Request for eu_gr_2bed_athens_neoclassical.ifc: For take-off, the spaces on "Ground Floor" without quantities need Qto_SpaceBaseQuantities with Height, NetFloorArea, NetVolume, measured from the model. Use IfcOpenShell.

First a look at what the model holds.

```python
import ifcopenshell
import ifcopenshell.util.element
import ifcopenshell.util.unit

model = ifcopenshell.open("eu_gr_2bed_athens_neoclassical.ifc")
print(model.schema)
for unit_type in ("LENGTHUNIT", "AREAUNIT", "VOLUMEUNIT"):
    print(unit_type, ifcopenshell.util.unit.calculate_unit_scale(model, unit_type))
storey = next(s for s in model.by_type("IfcBuildingStorey") if s.Name == "Ground Floor")
spaces = [e for e in ifcopenshell.util.element.get_decomposition(storey) if e.is_a("IfcSpace")]
for e in sorted(spaces, key=lambda e: e.id()):
    print(e.id(), e.is_a(), e.Name, list(ifcopenshell.util.element.get_psets(e, qtos_only=True)), sep=" | ")
```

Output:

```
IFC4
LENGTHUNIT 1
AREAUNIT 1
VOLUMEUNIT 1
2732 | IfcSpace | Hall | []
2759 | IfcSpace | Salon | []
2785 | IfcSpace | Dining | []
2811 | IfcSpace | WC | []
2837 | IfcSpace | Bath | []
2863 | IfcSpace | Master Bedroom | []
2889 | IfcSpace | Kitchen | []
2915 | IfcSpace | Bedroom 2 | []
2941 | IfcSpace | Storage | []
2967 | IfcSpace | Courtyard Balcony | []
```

```python
import ifcopenshell
import ifcopenshell.api.pset
import ifcopenshell.geom
import ifcopenshell.util.element
import ifcopenshell.util.shape
import ifcopenshell.util.unit

model = ifcopenshell.open("eu_gr_2bed_athens_neoclassical.ifc")
unit_scale = ifcopenshell.util.unit.calculate_unit_scale(model)
area_scale = ifcopenshell.util.unit.calculate_unit_scale(model, "AREAUNIT")
volume_scale = ifcopenshell.util.unit.calculate_unit_scale(model, "VOLUMEUNIT")
settings = ifcopenshell.geom.settings()

storey = next(s for s in model.by_type("IfcBuildingStorey") if s.Name == "Ground Floor")
spaces = [e for e in ifcopenshell.util.element.get_decomposition(storey) if e.is_a("IfcSpace")]

for e in sorted(spaces, key=lambda e: e.id()):
    if ifcopenshell.util.element.get_psets(e, qtos_only=True, should_inherit=False):
        continue
    # Geometry comes back in metres, in the element's own axes.
    shape = ifcopenshell.geom.create_shape(settings, e)
    values = {
        "Height": ifcopenshell.util.shape.get_z(shape.geometry) / unit_scale,
        "NetFloorArea": ifcopenshell.util.shape.get_footprint_area(shape.geometry) / area_scale,
        "NetVolume": ifcopenshell.util.shape.get_volume(shape.geometry) / volume_scale,
    }
    qto = ifcopenshell.api.pset.add_qto(model, product=e, name="Qto_SpaceBaseQuantities")
    ifcopenshell.api.pset.edit_qto(model, qto=qto, properties=values)
    print(e.id(), {k: round(v, 3) for k, v in values.items()})

model.write("eu_gr_2bed_athens_neoclassical_v2.ifc")
```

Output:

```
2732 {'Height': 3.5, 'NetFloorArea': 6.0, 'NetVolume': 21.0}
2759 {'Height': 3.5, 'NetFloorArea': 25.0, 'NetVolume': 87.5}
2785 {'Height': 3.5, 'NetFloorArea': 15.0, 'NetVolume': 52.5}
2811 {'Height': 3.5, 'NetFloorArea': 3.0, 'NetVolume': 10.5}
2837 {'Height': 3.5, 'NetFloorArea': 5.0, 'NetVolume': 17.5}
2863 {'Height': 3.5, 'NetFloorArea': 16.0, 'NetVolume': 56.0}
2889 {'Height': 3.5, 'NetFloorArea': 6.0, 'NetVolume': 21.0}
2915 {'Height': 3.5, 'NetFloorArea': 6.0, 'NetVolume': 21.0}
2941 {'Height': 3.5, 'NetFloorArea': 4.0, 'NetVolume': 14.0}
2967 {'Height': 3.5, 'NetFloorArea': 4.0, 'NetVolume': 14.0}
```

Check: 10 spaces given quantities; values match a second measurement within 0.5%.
